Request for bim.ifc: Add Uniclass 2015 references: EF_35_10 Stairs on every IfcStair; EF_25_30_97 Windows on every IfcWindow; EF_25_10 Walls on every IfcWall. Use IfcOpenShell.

First a look at what the model holds.

```python
import ifcopenshell

model = ifcopenshell.open("bim.ifc")
print(model.schema)
print("classifications:", [c.Name for c in model.by_type("IfcClassification")])
for ifc_class in ("IfcDoor", "IfcRoof", "IfcStair", "IfcWall", "IfcWindow"):
    print(ifc_class, len(model.by_type(ifc_class)))
```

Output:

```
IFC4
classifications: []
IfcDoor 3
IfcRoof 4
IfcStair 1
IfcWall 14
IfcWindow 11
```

```python
import ifcopenshell
import ifcopenshell.api.classification

model = ifcopenshell.open("bim.ifc")

system = ifcopenshell.api.classification.add_classification(model, classification="Uniclass 2015")

codes = {
    "IfcStair": ("EF_35_10", "Stairs"),
    "IfcWindow": ("EF_25_30_97", "Windows"),
    "IfcWall": ("EF_25_10", "Walls"),
}
for ifc_class, (code, name) in codes.items():
    products = model.by_type(ifc_class)
    ifcopenshell.api.classification.add_reference(
        model, products=products, classification=system, identification=code, name=name
    )
    print(code, len(products))

model.write("bim_v2.ifc")
```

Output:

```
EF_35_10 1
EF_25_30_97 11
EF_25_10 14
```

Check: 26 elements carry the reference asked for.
